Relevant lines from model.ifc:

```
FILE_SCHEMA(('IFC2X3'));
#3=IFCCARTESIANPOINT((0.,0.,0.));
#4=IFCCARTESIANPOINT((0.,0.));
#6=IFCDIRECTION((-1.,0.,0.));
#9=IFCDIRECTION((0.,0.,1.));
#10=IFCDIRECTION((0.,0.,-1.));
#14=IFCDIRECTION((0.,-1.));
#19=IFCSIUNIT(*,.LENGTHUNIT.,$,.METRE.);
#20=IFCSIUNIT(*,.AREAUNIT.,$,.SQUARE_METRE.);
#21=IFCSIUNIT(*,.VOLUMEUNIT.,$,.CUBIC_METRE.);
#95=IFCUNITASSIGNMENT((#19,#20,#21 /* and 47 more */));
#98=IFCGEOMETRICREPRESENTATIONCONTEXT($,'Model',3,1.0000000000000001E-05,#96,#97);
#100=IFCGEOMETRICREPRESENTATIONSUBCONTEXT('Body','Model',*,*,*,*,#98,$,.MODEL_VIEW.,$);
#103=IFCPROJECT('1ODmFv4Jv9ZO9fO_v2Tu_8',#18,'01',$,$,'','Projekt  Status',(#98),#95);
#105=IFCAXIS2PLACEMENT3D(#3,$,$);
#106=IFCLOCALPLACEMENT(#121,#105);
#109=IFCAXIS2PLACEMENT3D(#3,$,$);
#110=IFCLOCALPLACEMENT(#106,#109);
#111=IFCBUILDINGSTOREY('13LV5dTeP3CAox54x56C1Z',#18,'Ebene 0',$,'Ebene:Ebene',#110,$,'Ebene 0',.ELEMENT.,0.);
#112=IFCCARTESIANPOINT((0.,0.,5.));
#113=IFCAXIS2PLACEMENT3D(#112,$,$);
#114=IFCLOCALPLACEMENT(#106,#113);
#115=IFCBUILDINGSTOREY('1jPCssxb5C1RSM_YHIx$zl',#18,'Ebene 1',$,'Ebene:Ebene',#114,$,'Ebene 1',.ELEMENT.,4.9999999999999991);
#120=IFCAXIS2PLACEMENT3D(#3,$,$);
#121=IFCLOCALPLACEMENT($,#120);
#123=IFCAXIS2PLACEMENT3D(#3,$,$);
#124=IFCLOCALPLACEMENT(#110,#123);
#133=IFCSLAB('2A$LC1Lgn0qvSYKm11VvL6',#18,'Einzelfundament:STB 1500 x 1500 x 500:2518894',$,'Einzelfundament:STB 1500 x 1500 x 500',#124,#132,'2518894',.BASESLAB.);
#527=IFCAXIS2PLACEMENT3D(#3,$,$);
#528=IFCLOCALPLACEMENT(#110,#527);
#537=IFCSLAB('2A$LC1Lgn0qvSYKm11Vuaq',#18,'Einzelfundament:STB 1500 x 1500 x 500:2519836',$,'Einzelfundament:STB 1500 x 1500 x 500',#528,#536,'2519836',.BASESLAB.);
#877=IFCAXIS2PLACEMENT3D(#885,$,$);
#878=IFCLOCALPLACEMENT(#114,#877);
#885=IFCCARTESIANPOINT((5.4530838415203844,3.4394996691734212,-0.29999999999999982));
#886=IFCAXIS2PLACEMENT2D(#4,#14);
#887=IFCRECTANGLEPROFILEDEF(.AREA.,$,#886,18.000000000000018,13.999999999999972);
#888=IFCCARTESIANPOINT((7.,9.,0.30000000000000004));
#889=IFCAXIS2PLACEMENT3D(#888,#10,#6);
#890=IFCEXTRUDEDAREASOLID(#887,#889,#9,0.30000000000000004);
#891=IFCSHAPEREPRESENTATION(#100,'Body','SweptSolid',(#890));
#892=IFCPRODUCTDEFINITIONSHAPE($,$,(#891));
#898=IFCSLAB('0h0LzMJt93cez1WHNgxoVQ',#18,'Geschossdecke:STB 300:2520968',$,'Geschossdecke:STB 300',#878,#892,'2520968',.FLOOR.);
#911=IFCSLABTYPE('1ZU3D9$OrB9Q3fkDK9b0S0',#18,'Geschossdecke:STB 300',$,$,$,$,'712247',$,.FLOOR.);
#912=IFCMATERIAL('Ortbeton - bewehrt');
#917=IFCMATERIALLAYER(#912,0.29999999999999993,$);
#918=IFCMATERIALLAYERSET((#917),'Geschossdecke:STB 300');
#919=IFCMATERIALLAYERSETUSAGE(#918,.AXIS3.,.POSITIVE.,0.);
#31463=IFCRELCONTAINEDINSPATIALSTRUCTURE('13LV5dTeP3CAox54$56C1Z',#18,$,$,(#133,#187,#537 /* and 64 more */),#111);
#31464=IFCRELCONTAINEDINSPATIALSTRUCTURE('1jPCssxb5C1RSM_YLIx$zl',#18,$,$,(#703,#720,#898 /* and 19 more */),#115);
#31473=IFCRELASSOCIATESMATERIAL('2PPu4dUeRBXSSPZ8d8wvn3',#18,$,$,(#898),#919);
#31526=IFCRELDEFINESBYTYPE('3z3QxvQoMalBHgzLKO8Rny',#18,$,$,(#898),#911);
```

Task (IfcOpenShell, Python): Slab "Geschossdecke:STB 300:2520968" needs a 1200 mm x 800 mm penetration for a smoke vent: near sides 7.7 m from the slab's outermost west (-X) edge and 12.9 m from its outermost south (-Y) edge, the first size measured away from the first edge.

```python
import numpy as np
import ifcopenshell
import ifcopenshell.api.feature
import ifcopenshell.api.geometry
import ifcopenshell.api.root
import ifcopenshell.geom
import ifcopenshell.util.placement
import ifcopenshell.util.representation
import ifcopenshell.util.shape
import ifcopenshell.util.unit

model = ifcopenshell.open("model.ifc")
unit_scale = ifcopenshell.util.unit.calculate_unit_scale(model)
settings = ifcopenshell.geom.settings()


def volume(element):
    """Net volume in cubic metres, openings subtracted."""
    shape = ifcopenshell.geom.create_shape(settings, element)
    return ifcopenshell.util.shape.get_volume(shape.geometry)


slab = model.by_guid("0h0LzMJt93cez1WHNgxoVQ")
before = volume(slab)

# Extent in the slab's own axes, in metres. The edges named are its -X and -Y sides.
slab_shape = ifcopenshell.geom.create_shape(settings, slab)
vertices = ifcopenshell.util.shape.get_vertices(slab_shape.geometry)
x_min, y_min, bottom = vertices.min(axis=0)
top = vertices[:, 2].max()

opening = ifcopenshell.api.root.create_entity(model, ifc_class="IfcOpeningElement", name="Smoke vent opening")
context = ifcopenshell.util.representation.get_context(model, "Model", "Body", "MODEL_VIEW")
width, depth = 1.2, 0.8
outline = [(0.0, 0.0), (width, 0.0), (width, depth), (0.0, depth), (0.0, 0.0)]
# Overshoot both faces by 50 mm so the cut is clean.
shape = ifcopenshell.api.geometry.add_slab_representation(
    model, context=context, depth=top - bottom + 0.1, polyline=outline
)
ifcopenshell.api.geometry.assign_representation(model, product=opening, representation=shape)

matrix = ifcopenshell.util.placement.get_local_placement(slab.ObjectPlacement)
matrix[:, 3] = matrix @ np.append(np.array([x_min + 7.7, y_min + 12.9, bottom - 0.05]) / unit_scale, 1.0)
ifcopenshell.api.geometry.edit_object_placement(model, product=opening, matrix=matrix, is_si=False)
ifcopenshell.api.feature.add_feature(model, feature=opening, element=slab)

after = volume(slab)

print(f"slab volume {before:.3f} -> {after:.3f} m3")

model.write("model_edited.ifc")
```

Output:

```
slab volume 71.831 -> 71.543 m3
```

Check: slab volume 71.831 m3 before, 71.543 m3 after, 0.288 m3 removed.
